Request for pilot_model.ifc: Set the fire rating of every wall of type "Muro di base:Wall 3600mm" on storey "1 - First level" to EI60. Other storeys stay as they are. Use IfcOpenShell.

First a look at what the model holds.

```python
import ifcopenshell
import ifcopenshell.util.element

model = ifcopenshell.open("pilot_model.ifc")
print(model.schema)
storey = next(s for s in model.by_type("IfcBuildingStorey") if s.Name == "1 - First level")
walls = [e for e in ifcopenshell.util.element.get_decomposition(storey) if e.is_a("IfcWall")]
seen = {}
for e in walls:
    element_type = ifcopenshell.util.element.get_type(e)
    key = (element_type.Name if element_type != e and element_type else None, ifcopenshell.util.element.get_pset(e, "Pset_WallCommon", "FireRating"))
    seen[key] = seen.get(key, 0) + 1
for (name, value), count in sorted(seen.items(), key=str):
    print(count, "x", name, "|", value)
```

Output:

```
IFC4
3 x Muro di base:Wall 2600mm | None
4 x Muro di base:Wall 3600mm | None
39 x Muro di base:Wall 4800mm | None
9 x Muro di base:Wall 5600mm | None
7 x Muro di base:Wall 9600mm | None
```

```python
import ifcopenshell
import ifcopenshell.api.pset
import ifcopenshell.util.element

model = ifcopenshell.open("pilot_model.ifc")

storey = next(s for s in model.by_type("IfcBuildingStorey") if s.Name == "1 - First level")
walls = [e for e in ifcopenshell.util.element.get_decomposition(storey) if e.is_a("IfcWall")]

count = 0
for e in walls:
    element_type = ifcopenshell.util.element.get_type(e)
    if element_type in (None, e) or element_type.Name != "Muro di base:Wall 3600mm":
        continue
    # add_pset returns the element's existing set when there is one.
    pset = ifcopenshell.api.pset.add_pset(model, product=e, name="Pset_WallCommon")
    ifcopenshell.api.pset.edit_pset(model, pset=pset, properties={"FireRating": "EI60"})
    count += 1

print(count, "walls updated")

model.write("pilot_model-out.ifc")
```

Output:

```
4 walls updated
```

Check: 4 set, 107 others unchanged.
